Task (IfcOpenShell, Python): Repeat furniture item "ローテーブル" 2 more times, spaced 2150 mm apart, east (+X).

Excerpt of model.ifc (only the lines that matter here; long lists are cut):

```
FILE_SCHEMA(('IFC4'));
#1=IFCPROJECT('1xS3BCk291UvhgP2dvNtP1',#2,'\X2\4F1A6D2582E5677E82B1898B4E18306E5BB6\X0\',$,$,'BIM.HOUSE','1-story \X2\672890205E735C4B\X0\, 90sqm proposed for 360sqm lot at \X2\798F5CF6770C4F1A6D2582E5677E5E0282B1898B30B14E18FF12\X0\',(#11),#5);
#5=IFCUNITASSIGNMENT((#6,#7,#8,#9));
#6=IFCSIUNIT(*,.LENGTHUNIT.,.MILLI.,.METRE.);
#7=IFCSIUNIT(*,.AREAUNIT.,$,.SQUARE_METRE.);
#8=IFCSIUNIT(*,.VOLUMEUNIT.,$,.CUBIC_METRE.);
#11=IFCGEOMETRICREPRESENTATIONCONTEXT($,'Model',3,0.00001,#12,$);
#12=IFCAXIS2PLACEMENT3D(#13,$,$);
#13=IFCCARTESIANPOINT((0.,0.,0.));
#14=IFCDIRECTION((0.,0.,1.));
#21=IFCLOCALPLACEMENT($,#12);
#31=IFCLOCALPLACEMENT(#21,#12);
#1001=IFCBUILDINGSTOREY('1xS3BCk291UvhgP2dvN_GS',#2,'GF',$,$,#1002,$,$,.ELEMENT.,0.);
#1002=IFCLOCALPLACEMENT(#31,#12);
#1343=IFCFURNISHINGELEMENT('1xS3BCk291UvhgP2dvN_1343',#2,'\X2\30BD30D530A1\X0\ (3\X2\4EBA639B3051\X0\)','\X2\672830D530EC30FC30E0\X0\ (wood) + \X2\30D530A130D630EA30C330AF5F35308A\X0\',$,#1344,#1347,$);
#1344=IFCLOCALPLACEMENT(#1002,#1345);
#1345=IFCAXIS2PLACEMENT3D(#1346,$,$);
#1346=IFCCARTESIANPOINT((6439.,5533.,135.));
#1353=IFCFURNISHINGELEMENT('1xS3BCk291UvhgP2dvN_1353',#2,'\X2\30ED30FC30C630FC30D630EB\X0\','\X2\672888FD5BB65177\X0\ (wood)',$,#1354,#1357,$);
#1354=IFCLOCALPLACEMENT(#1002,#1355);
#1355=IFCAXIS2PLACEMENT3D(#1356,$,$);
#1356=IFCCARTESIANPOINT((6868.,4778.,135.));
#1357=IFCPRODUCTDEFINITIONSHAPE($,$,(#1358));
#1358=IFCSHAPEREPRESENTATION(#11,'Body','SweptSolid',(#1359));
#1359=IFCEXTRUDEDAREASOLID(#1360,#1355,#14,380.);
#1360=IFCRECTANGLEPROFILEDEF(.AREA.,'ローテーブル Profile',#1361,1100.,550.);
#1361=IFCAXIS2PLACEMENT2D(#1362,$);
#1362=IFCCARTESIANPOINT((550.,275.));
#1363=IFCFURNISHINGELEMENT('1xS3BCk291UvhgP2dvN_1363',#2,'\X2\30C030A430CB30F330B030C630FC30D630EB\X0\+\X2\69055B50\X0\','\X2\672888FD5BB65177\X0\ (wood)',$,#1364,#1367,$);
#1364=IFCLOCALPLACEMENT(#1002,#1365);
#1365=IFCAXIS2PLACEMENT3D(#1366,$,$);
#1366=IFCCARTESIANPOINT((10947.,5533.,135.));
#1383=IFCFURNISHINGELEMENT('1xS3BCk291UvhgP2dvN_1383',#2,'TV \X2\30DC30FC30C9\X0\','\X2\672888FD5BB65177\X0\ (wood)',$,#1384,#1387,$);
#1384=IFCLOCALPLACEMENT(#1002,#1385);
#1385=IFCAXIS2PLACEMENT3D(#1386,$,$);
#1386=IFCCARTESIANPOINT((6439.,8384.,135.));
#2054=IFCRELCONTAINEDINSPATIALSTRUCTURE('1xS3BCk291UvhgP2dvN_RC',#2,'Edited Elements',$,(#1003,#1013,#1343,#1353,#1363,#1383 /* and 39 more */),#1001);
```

```python
import numpy as np
import ifcopenshell
import ifcopenshell.api.geometry
import ifcopenshell.api.root
import ifcopenshell.util.element
import ifcopenshell.util.placement

model = ifcopenshell.open("model.ifc")


def reuse_history(source, copy):
    """copy_class also copies each property set's owner history, people and application; keep the originals."""
    for rel in copy.IsDefinedBy:
        if rel.is_a("IfcRelDefinesByProperties") and (history := rel.RelatingPropertyDefinition.OwnerHistory):
            rel.RelatingPropertyDefinition.OwnerHistory = source.OwnerHistory
            ifcopenshell.util.element.remove_deep2(model, history)


source = model.by_id(1353)
base = ifcopenshell.util.placement.get_local_placement(source.ObjectPlacement)
step = np.array([1.0, 0.0, 0.0]) * 2150.0

for i in range(1, 3):
    copy = ifcopenshell.api.root.copy_class(model, product=source)
    copy.Representation = ifcopenshell.util.element.copy_deep(
        model, source.Representation, exclude=["IfcGeometricRepresentationContext", "IfcRepresentationMap"]
    )
    reuse_history(source, copy)
    matrix = base.copy()
    matrix[:3, 3] += i * step
    print("added at", matrix[:3, 3].round(3) + 0.0)
    ifcopenshell.api.geometry.edit_object_placement(model, product=copy, matrix=matrix, is_si=False)

model.write("model_v2.ifc")
```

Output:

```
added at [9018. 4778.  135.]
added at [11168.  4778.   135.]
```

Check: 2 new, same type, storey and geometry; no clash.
